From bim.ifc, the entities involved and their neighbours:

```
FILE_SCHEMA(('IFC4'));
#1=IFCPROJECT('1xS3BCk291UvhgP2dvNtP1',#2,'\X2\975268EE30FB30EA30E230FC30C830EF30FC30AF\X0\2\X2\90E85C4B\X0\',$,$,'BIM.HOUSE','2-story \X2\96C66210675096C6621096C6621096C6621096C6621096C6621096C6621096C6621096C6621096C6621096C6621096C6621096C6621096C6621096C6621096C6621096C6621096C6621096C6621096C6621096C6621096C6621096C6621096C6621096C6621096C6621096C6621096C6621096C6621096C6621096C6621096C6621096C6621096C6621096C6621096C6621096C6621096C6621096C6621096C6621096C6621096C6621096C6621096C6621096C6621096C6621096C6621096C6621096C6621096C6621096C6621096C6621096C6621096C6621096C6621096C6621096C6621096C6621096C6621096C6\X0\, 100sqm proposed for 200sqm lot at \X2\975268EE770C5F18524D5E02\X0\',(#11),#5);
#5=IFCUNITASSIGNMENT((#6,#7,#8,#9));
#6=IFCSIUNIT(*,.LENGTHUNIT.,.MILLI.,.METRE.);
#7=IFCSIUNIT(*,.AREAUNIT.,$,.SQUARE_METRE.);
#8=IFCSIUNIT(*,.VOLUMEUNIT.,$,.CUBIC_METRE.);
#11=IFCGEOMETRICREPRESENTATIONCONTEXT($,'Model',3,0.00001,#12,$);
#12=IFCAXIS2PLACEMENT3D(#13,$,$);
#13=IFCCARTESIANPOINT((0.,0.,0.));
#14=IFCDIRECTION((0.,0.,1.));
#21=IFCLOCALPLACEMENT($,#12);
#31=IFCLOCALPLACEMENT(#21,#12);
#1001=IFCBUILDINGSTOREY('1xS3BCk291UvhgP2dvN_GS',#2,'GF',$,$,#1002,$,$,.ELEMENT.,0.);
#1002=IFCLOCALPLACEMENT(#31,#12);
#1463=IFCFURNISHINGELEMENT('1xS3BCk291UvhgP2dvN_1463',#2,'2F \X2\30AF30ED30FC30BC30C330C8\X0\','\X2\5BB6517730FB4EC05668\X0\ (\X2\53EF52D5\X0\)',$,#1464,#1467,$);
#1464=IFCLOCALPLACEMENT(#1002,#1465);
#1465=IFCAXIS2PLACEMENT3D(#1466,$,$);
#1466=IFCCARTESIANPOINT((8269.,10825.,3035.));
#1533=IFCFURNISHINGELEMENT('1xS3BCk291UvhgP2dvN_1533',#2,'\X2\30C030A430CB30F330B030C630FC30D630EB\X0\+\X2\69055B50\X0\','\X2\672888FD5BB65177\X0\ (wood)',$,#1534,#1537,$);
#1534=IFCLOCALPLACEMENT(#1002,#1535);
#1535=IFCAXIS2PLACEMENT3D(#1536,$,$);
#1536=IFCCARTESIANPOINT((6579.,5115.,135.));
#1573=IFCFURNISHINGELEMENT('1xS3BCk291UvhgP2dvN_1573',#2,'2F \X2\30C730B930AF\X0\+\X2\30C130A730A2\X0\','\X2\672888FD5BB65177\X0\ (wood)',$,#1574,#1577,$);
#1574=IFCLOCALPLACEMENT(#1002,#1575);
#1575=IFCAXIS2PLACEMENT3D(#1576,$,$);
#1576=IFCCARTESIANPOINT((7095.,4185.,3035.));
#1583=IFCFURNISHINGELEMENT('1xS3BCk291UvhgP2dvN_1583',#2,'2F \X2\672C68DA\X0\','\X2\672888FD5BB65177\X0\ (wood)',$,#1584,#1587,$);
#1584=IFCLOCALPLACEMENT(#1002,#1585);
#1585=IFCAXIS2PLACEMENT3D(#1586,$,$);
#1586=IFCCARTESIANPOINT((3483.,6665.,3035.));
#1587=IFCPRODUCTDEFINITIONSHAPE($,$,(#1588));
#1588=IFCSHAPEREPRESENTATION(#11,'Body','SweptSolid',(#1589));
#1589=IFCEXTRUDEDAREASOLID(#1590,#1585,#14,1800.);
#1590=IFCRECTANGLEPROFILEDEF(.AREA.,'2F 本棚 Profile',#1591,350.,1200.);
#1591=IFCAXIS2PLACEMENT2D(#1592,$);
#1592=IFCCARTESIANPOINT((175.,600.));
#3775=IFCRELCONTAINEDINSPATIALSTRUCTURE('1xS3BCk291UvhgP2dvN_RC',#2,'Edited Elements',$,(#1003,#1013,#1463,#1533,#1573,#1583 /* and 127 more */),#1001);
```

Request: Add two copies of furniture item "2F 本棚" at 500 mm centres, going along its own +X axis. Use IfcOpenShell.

```python
import ifcopenshell
import ifcopenshell.api.geometry
import ifcopenshell.api.root
import ifcopenshell.util.element
import ifcopenshell.util.placement
import ifcopenshell.util.unit

model = ifcopenshell.open("bim.ifc")
unit_scale = ifcopenshell.util.unit.calculate_unit_scale(model)


def reuse_history(source, copy):
    """copy_class also copies each property set's owner history, people and application; keep the originals."""
    for rel in copy.IsDefinedBy:
        if rel.is_a("IfcRelDefinesByProperties") and (history := rel.RelatingPropertyDefinition.OwnerHistory):
            rel.RelatingPropertyDefinition.OwnerHistory = source.OwnerHistory
            ifcopenshell.util.element.remove_deep2(model, history)


source = model.by_guid("1xS3BCk291UvhgP2dvN_1583")
base = ifcopenshell.util.placement.get_local_placement(source.ObjectPlacement)
step = base[:3, 0] * 0.5 / unit_scale

for i in range(1, 3):
    copy = ifcopenshell.api.root.copy_class(model, product=source)
    copy.Representation = ifcopenshell.util.element.copy_deep(
        model, source.Representation, exclude=["IfcGeometricRepresentationContext", "IfcRepresentationMap"]
    )
    reuse_history(source, copy)
    matrix = base.copy()
    matrix[:3, 3] += i * step
    print("added at", matrix[:3, 3].round(3) + 0.0)
    ifcopenshell.api.geometry.edit_object_placement(model, product=copy, matrix=matrix, is_si=False)

model.write("bim_edited.ifc")
```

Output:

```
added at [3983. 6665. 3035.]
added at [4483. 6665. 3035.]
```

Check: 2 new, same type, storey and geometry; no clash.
